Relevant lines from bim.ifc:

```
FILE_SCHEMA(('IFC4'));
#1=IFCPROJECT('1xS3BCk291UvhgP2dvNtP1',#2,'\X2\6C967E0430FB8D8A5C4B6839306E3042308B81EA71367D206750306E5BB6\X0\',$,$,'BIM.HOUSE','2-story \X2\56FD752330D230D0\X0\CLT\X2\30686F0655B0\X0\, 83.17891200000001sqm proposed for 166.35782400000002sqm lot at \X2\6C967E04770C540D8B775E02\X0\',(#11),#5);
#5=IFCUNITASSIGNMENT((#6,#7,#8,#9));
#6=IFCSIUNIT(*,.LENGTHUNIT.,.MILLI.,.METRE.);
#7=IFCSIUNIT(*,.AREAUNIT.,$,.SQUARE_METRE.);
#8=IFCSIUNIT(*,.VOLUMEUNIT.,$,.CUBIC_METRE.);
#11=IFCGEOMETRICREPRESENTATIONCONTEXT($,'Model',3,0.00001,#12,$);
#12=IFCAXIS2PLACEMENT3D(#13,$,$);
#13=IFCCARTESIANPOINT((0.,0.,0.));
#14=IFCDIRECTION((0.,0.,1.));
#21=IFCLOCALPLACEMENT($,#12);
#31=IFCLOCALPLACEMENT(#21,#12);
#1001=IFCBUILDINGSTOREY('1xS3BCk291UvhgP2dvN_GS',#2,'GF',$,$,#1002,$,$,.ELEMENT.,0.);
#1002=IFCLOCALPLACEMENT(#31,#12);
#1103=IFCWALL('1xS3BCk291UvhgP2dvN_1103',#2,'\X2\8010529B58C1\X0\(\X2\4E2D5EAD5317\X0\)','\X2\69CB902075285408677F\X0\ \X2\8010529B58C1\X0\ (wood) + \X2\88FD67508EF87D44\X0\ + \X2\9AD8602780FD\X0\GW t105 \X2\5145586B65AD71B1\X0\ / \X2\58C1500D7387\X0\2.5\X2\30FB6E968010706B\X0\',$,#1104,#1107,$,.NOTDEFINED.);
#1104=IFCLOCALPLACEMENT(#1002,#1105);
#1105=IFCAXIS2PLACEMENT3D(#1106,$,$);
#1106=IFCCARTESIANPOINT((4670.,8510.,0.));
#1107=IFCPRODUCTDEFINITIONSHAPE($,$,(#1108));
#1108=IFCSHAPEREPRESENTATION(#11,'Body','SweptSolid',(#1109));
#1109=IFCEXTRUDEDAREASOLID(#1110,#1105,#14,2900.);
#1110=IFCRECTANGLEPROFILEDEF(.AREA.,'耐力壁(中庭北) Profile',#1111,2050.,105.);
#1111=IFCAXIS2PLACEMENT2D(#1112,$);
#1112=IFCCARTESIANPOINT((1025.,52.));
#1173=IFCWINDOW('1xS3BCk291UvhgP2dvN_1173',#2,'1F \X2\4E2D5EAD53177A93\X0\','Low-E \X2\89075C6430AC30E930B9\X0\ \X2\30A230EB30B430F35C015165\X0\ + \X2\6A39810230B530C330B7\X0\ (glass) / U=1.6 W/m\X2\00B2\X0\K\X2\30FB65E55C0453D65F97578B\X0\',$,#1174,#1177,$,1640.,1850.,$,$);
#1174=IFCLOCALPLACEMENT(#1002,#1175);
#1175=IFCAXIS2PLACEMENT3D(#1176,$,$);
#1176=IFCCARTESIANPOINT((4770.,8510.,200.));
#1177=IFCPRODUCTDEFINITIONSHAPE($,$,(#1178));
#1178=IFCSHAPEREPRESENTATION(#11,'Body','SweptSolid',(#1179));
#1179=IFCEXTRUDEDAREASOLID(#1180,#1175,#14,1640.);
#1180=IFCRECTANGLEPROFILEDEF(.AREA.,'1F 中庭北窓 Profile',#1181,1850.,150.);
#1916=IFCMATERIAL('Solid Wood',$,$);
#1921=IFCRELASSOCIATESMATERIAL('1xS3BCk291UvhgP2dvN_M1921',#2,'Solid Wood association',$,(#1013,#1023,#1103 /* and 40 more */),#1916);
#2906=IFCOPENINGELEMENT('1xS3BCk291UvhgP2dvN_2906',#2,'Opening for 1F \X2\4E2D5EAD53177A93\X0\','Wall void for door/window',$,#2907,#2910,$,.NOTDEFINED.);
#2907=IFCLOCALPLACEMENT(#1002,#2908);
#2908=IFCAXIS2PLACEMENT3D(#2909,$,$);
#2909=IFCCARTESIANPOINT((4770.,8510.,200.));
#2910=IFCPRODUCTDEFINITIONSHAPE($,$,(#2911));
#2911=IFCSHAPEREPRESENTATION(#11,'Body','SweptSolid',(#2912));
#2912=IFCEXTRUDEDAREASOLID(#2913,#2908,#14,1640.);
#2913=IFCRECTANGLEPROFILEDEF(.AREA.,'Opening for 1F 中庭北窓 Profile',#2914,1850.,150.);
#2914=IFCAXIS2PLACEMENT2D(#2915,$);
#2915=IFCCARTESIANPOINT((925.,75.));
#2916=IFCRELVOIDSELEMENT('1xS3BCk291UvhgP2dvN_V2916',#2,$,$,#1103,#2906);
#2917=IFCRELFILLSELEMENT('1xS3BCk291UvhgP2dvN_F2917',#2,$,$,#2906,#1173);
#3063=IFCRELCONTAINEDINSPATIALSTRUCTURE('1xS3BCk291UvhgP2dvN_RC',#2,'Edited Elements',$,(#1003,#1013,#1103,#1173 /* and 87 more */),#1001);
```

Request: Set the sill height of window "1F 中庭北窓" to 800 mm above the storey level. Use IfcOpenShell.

```python
import numpy as np
import ifcopenshell
import ifcopenshell.api.geometry
import ifcopenshell.geom
import ifcopenshell.util.element
import ifcopenshell.util.placement
import ifcopenshell.util.shape
import ifcopenshell.util.unit

model = ifcopenshell.open("bim.ifc")
unit_scale = ifcopenshell.util.unit.calculate_unit_scale(model)

window = model.by_id(1173)
opening = window.FillsVoids[0].RelatingOpeningElement
storey = ifcopenshell.util.element.get_container(window, ifc_class="IfcBuildingStorey")
level = ifcopenshell.util.placement.get_local_placement(storey.ObjectPlacement)[2, 3]

# The opening's origin need not be at the sill, so measure its lowest point.
shape = ifcopenshell.geom.create_shape(ifcopenshell.geom.settings(), opening)
bottom = ifcopenshell.util.shape.get_shape_bottom_elevation(shape, shape.geometry) / unit_scale
dz = level + 0.8 / unit_scale - bottom

shift = np.array([0.0, 0.0, dz])
# The window is not placed relative to its opening, so move both.
for product in (opening, window):
    matrix = ifcopenshell.util.placement.get_local_placement(product.ObjectPlacement)
    matrix[:3, 3] += shift
    ifcopenshell.api.geometry.edit_object_placement(model, product=product, matrix=matrix, is_si=False)

print(f"moved by {dz * unit_scale:+.3f} m")

model.write("bim_v2.ifc")
```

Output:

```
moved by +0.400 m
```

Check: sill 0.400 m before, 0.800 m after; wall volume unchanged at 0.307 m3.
